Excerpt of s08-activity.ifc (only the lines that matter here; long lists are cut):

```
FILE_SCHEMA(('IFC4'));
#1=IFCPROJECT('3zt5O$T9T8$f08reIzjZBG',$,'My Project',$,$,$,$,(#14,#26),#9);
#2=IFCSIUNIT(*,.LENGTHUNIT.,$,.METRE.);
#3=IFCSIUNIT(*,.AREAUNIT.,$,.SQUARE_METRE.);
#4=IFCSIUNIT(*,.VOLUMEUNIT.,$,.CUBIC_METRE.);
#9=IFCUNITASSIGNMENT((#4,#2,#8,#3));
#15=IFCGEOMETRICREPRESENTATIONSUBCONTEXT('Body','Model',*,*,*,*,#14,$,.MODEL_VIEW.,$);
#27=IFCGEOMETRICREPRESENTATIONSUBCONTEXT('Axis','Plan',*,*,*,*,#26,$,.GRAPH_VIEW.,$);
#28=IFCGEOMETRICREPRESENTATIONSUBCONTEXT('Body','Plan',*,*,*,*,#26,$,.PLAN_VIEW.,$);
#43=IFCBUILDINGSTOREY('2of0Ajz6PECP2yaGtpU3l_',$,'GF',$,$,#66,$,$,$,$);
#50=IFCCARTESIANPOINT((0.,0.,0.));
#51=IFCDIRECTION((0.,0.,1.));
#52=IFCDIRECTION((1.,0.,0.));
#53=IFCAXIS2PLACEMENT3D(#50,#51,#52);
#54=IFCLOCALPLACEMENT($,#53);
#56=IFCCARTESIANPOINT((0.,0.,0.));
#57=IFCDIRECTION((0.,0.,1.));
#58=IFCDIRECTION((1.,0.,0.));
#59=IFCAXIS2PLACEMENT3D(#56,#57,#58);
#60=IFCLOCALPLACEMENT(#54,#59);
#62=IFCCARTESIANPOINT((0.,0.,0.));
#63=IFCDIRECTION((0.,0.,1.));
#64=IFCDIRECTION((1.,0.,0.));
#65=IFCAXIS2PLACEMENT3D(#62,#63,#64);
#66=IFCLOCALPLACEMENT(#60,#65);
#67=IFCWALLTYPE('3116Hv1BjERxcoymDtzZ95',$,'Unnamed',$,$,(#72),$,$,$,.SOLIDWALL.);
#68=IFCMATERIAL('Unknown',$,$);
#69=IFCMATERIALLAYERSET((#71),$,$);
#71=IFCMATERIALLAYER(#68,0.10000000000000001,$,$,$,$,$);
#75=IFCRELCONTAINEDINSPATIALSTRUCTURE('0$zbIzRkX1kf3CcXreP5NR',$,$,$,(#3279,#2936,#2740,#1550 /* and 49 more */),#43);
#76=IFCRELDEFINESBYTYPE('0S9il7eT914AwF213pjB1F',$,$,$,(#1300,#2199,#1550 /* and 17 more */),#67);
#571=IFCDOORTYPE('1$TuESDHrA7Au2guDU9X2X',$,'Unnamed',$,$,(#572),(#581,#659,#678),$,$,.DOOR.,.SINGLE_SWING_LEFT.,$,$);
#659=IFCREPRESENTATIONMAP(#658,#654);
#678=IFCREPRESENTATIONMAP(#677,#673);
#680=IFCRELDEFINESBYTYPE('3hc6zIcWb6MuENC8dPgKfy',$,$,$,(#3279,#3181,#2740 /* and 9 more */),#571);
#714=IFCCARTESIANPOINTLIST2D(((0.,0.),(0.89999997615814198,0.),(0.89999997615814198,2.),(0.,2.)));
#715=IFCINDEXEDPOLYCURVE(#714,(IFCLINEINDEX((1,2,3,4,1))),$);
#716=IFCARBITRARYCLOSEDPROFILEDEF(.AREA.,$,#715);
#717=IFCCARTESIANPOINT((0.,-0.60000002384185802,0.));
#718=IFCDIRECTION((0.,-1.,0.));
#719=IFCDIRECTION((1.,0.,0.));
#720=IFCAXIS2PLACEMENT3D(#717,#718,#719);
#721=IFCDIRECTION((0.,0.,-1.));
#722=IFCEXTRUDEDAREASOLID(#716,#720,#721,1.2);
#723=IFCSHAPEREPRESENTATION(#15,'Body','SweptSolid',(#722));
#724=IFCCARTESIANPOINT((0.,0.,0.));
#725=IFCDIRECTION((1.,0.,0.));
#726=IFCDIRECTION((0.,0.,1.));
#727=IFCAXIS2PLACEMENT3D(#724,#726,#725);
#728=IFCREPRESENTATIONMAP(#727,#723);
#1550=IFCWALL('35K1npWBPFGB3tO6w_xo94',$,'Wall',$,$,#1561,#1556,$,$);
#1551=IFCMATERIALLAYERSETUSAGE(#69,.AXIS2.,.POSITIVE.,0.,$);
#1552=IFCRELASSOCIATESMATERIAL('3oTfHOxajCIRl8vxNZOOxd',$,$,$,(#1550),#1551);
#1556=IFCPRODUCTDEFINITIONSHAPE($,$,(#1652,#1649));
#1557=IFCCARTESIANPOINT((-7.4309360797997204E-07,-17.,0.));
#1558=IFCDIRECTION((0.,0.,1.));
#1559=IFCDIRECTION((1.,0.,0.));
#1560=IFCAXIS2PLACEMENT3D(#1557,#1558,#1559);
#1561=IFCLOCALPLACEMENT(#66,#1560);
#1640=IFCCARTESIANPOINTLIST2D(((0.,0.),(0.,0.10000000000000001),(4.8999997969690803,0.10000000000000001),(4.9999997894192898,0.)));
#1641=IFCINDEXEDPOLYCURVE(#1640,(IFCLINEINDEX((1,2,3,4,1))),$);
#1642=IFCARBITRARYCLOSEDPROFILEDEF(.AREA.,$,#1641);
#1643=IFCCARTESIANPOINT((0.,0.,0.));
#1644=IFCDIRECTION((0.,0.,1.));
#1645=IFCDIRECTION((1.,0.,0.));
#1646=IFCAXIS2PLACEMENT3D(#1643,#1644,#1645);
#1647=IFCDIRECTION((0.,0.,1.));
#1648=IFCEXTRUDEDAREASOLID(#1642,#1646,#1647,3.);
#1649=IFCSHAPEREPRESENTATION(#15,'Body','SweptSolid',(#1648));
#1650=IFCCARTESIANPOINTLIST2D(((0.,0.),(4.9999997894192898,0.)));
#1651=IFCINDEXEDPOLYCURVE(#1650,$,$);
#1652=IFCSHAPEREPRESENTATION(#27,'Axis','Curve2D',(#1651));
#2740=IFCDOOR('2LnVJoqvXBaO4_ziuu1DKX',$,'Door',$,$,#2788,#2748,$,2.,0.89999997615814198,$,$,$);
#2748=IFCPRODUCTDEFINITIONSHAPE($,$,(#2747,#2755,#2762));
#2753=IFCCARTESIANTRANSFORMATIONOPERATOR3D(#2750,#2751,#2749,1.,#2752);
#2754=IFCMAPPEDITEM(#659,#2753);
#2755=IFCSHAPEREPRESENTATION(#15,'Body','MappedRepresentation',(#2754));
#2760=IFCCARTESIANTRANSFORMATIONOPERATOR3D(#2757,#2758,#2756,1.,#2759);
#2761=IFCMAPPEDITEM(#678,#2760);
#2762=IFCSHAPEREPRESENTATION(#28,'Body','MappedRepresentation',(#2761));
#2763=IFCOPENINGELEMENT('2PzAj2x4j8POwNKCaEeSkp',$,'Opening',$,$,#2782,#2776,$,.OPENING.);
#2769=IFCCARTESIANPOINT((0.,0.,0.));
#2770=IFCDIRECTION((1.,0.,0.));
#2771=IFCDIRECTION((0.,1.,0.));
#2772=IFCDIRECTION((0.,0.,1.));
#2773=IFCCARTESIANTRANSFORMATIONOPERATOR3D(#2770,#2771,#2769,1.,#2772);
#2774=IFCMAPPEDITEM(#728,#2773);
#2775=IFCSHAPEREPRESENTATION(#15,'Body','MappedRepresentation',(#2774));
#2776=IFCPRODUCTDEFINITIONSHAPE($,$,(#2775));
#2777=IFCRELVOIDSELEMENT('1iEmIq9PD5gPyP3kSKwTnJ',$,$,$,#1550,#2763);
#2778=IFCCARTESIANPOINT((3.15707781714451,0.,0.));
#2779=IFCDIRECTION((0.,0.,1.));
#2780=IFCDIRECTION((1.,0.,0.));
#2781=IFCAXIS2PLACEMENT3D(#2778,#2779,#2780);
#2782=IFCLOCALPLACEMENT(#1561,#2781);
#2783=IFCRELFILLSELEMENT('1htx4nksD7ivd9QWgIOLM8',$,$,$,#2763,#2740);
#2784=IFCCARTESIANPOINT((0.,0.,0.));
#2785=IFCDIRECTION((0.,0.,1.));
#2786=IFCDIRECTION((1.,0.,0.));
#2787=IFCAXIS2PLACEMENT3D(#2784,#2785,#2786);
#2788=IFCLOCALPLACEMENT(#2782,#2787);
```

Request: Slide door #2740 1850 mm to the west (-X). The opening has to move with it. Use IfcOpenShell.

```python
import ifcopenshell
import ifcopenshell.api.geometry
import ifcopenshell.util.placement
import ifcopenshell.util.unit

model = ifcopenshell.open("s08-activity.ifc")
unit_scale = ifcopenshell.util.unit.calculate_unit_scale(model)

door = model.by_guid("2LnVJoqvXBaO4_ziuu1DKX")
opening = door.FillsVoids[0].RelatingOpeningElement
wall = opening.VoidsElements[0].RelatingBuildingElement

wall_matrix = ifcopenshell.util.placement.get_local_placement(wall.ObjectPlacement)
shift = wall_matrix[:3, 0] * -1.85 / unit_scale
before = ifcopenshell.util.placement.get_local_placement(door.ObjectPlacement)[:3, 3].copy()

# The door is placed relative to its opening, so it follows when the opening moves.
matrix = ifcopenshell.util.placement.get_local_placement(opening.ObjectPlacement)
matrix[:3, 3] += shift
ifcopenshell.api.geometry.edit_object_placement(
    model, product=opening, matrix=matrix, is_si=False, should_transform_children=True
)

after = ifcopenshell.util.placement.get_local_placement(door.ObjectPlacement)[:3, 3]
print("door moved by", (after - before).round(3) + 0.0)

model.write("s08-activity_edited.ifc")
```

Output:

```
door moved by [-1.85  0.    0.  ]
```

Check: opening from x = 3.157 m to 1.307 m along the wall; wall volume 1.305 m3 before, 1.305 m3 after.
